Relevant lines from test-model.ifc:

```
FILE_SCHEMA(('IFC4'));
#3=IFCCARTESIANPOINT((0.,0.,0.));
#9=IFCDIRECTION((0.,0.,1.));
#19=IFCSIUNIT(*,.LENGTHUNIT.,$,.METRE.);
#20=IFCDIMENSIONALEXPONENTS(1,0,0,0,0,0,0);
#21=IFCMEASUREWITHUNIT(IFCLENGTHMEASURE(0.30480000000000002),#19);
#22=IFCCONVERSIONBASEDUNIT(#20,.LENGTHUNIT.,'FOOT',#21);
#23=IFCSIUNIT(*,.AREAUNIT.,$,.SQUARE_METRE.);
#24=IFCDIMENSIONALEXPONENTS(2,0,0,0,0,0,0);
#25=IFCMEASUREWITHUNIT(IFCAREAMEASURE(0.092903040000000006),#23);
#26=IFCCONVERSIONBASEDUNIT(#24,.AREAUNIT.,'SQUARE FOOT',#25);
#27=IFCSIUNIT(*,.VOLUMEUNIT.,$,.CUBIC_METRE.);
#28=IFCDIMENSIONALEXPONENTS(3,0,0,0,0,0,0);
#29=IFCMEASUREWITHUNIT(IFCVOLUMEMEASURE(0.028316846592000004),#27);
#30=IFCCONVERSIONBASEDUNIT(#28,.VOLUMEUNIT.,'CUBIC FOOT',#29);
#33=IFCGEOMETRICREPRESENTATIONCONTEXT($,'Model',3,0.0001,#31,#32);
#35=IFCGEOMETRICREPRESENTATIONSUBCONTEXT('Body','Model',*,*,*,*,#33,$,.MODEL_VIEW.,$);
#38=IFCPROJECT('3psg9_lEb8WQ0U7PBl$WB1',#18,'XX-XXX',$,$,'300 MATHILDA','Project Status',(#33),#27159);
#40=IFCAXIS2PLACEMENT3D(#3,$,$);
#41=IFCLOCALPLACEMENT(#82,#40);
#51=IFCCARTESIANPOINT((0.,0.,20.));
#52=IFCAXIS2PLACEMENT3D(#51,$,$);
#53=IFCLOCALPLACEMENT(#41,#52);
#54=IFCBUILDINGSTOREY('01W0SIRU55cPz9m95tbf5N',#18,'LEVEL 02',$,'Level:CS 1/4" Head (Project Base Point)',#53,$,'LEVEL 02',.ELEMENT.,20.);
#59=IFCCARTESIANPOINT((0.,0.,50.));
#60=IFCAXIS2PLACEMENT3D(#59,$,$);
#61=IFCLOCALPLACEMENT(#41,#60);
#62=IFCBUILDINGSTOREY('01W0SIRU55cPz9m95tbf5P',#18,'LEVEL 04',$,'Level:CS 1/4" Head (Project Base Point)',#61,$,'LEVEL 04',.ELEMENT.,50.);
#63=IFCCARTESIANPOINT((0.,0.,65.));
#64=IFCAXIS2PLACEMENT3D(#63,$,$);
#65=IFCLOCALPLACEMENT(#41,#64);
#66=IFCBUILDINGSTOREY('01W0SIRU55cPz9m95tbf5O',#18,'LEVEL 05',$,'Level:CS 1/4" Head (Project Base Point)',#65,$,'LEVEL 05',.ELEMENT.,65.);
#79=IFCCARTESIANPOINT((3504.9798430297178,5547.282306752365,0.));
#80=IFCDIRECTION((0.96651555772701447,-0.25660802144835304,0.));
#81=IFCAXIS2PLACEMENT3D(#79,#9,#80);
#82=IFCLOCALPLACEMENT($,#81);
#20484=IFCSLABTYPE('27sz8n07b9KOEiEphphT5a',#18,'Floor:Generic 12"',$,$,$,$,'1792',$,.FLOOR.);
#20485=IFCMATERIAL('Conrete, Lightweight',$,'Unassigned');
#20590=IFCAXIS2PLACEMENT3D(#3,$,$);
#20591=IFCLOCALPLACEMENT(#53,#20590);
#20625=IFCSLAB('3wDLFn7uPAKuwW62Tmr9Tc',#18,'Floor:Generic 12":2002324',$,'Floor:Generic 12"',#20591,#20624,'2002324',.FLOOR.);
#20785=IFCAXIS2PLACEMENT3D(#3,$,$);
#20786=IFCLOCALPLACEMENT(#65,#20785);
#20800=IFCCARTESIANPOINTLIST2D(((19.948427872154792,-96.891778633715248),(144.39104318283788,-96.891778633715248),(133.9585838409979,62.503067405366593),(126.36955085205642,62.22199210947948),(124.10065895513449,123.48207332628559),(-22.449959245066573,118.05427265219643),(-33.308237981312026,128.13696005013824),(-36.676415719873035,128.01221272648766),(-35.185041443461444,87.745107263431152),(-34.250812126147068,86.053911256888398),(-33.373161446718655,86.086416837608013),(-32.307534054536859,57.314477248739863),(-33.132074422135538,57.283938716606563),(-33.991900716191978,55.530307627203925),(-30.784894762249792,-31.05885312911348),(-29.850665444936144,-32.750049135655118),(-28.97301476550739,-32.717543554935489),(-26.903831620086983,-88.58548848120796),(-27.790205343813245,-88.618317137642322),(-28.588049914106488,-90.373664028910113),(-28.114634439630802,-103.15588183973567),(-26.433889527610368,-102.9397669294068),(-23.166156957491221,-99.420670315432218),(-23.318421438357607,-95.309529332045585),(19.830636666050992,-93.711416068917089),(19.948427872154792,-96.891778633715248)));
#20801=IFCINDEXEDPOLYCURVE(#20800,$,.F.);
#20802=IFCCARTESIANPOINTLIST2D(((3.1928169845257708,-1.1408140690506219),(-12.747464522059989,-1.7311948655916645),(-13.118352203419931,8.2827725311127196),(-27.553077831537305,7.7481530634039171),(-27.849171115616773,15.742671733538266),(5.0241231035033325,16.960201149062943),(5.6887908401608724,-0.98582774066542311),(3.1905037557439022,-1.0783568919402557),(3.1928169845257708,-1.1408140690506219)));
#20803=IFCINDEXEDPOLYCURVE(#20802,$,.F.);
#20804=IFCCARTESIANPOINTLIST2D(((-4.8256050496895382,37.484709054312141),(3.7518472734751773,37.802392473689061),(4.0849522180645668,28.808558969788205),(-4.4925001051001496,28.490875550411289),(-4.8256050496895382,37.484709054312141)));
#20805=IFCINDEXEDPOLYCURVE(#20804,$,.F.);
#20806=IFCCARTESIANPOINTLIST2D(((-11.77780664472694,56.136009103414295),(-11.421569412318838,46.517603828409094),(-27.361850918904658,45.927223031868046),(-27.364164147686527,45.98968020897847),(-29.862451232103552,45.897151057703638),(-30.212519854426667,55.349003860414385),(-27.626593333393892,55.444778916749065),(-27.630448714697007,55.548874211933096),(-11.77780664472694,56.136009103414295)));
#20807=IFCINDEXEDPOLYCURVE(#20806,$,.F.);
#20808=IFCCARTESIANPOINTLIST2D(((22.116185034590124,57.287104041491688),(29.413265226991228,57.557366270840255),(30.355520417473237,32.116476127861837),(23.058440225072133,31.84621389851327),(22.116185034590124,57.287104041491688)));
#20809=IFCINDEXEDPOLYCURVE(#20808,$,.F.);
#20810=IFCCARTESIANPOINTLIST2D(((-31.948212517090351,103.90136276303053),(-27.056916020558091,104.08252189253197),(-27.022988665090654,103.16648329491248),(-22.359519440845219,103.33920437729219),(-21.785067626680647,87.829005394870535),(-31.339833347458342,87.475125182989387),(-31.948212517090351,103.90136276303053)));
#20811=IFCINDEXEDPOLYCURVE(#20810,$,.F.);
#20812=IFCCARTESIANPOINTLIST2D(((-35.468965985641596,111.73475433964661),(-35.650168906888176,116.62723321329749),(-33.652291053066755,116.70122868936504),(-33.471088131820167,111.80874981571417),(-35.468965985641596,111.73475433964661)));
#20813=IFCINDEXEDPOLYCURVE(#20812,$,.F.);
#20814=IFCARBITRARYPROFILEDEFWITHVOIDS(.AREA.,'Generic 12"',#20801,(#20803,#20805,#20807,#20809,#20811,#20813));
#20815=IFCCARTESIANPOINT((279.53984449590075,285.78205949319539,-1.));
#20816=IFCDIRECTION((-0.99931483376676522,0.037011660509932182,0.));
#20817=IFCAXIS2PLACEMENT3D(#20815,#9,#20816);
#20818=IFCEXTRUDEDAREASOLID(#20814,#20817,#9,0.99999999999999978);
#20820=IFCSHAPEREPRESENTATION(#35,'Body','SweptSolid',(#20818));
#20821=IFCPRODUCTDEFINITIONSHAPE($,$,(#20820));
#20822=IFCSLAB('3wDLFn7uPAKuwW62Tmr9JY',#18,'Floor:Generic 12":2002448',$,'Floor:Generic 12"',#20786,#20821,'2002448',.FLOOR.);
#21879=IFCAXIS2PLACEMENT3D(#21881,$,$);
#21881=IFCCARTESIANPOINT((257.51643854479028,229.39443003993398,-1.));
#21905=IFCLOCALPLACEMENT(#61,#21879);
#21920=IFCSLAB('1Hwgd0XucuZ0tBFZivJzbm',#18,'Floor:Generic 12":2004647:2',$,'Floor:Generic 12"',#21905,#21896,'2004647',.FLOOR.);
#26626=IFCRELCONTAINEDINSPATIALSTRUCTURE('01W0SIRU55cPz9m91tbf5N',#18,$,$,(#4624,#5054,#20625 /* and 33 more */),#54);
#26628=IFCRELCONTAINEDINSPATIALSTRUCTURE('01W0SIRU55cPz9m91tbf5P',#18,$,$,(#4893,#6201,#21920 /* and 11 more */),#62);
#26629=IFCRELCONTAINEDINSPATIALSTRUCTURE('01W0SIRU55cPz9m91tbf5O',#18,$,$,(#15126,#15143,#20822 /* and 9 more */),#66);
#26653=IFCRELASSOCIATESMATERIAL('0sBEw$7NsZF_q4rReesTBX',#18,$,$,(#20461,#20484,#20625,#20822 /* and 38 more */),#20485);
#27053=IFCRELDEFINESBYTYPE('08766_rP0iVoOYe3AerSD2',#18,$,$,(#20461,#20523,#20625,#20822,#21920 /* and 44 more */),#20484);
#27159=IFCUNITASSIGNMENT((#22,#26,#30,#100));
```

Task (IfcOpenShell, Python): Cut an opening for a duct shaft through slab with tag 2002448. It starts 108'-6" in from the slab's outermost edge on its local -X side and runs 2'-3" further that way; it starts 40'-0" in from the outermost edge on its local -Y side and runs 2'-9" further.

```python
import numpy as np
import ifcopenshell
import ifcopenshell.api.feature
import ifcopenshell.api.geometry
import ifcopenshell.api.root
import ifcopenshell.geom
import ifcopenshell.util.placement
import ifcopenshell.util.representation
import ifcopenshell.util.shape
import ifcopenshell.util.unit

model = ifcopenshell.open("test-model.ifc")
unit_scale = ifcopenshell.util.unit.calculate_unit_scale(model)
settings = ifcopenshell.geom.settings()


def volume(element):
    """Net volume in cubic metres, openings subtracted."""
    shape = ifcopenshell.geom.create_shape(settings, element)
    return ifcopenshell.util.shape.get_volume(shape.geometry)


slab = model.by_guid("3wDLFn7uPAKuwW62Tmr9JY")
before = volume(slab)

# Extent in the slab's own axes, in metres. The edges named are its -X and -Y sides.
slab_shape = ifcopenshell.geom.create_shape(settings, slab)
vertices = ifcopenshell.util.shape.get_vertices(slab_shape.geometry)
x_min, y_min, bottom = vertices.min(axis=0)
top = vertices[:, 2].max()

opening = ifcopenshell.api.root.create_entity(model, ifc_class="IfcOpeningElement", name="Duct shaft opening", predefined_type="OPENING")
context = ifcopenshell.util.representation.get_context(model, "Model", "Body", "MODEL_VIEW")
width, depth = 0.6858, 0.8382
outline = [(0.0, 0.0), (width, 0.0), (width, depth), (0.0, depth), (0.0, 0.0)]
# Overshoot both faces by 50 mm so the cut is clean.
shape = ifcopenshell.api.geometry.add_slab_representation(
    model, context=context, depth=top - bottom + 0.1, polyline=outline
)
ifcopenshell.api.geometry.assign_representation(model, product=opening, representation=shape)

matrix = ifcopenshell.util.placement.get_local_placement(slab.ObjectPlacement)
matrix[:, 3] = matrix @ np.append(np.array([x_min + 33.0708, y_min + 12.192, bottom - 0.05]) / unit_scale, 1.0)
ifcopenshell.api.geometry.edit_object_placement(model, product=opening, matrix=matrix, is_si=False)
ifcopenshell.api.feature.add_feature(model, feature=opening, element=slab)

after = volume(slab)

print(f"slab volume {before:.3f} -> {after:.3f} m3")

model.write("test-model_v2.ifc")
```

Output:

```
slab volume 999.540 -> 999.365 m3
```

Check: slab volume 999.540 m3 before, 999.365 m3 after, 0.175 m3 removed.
